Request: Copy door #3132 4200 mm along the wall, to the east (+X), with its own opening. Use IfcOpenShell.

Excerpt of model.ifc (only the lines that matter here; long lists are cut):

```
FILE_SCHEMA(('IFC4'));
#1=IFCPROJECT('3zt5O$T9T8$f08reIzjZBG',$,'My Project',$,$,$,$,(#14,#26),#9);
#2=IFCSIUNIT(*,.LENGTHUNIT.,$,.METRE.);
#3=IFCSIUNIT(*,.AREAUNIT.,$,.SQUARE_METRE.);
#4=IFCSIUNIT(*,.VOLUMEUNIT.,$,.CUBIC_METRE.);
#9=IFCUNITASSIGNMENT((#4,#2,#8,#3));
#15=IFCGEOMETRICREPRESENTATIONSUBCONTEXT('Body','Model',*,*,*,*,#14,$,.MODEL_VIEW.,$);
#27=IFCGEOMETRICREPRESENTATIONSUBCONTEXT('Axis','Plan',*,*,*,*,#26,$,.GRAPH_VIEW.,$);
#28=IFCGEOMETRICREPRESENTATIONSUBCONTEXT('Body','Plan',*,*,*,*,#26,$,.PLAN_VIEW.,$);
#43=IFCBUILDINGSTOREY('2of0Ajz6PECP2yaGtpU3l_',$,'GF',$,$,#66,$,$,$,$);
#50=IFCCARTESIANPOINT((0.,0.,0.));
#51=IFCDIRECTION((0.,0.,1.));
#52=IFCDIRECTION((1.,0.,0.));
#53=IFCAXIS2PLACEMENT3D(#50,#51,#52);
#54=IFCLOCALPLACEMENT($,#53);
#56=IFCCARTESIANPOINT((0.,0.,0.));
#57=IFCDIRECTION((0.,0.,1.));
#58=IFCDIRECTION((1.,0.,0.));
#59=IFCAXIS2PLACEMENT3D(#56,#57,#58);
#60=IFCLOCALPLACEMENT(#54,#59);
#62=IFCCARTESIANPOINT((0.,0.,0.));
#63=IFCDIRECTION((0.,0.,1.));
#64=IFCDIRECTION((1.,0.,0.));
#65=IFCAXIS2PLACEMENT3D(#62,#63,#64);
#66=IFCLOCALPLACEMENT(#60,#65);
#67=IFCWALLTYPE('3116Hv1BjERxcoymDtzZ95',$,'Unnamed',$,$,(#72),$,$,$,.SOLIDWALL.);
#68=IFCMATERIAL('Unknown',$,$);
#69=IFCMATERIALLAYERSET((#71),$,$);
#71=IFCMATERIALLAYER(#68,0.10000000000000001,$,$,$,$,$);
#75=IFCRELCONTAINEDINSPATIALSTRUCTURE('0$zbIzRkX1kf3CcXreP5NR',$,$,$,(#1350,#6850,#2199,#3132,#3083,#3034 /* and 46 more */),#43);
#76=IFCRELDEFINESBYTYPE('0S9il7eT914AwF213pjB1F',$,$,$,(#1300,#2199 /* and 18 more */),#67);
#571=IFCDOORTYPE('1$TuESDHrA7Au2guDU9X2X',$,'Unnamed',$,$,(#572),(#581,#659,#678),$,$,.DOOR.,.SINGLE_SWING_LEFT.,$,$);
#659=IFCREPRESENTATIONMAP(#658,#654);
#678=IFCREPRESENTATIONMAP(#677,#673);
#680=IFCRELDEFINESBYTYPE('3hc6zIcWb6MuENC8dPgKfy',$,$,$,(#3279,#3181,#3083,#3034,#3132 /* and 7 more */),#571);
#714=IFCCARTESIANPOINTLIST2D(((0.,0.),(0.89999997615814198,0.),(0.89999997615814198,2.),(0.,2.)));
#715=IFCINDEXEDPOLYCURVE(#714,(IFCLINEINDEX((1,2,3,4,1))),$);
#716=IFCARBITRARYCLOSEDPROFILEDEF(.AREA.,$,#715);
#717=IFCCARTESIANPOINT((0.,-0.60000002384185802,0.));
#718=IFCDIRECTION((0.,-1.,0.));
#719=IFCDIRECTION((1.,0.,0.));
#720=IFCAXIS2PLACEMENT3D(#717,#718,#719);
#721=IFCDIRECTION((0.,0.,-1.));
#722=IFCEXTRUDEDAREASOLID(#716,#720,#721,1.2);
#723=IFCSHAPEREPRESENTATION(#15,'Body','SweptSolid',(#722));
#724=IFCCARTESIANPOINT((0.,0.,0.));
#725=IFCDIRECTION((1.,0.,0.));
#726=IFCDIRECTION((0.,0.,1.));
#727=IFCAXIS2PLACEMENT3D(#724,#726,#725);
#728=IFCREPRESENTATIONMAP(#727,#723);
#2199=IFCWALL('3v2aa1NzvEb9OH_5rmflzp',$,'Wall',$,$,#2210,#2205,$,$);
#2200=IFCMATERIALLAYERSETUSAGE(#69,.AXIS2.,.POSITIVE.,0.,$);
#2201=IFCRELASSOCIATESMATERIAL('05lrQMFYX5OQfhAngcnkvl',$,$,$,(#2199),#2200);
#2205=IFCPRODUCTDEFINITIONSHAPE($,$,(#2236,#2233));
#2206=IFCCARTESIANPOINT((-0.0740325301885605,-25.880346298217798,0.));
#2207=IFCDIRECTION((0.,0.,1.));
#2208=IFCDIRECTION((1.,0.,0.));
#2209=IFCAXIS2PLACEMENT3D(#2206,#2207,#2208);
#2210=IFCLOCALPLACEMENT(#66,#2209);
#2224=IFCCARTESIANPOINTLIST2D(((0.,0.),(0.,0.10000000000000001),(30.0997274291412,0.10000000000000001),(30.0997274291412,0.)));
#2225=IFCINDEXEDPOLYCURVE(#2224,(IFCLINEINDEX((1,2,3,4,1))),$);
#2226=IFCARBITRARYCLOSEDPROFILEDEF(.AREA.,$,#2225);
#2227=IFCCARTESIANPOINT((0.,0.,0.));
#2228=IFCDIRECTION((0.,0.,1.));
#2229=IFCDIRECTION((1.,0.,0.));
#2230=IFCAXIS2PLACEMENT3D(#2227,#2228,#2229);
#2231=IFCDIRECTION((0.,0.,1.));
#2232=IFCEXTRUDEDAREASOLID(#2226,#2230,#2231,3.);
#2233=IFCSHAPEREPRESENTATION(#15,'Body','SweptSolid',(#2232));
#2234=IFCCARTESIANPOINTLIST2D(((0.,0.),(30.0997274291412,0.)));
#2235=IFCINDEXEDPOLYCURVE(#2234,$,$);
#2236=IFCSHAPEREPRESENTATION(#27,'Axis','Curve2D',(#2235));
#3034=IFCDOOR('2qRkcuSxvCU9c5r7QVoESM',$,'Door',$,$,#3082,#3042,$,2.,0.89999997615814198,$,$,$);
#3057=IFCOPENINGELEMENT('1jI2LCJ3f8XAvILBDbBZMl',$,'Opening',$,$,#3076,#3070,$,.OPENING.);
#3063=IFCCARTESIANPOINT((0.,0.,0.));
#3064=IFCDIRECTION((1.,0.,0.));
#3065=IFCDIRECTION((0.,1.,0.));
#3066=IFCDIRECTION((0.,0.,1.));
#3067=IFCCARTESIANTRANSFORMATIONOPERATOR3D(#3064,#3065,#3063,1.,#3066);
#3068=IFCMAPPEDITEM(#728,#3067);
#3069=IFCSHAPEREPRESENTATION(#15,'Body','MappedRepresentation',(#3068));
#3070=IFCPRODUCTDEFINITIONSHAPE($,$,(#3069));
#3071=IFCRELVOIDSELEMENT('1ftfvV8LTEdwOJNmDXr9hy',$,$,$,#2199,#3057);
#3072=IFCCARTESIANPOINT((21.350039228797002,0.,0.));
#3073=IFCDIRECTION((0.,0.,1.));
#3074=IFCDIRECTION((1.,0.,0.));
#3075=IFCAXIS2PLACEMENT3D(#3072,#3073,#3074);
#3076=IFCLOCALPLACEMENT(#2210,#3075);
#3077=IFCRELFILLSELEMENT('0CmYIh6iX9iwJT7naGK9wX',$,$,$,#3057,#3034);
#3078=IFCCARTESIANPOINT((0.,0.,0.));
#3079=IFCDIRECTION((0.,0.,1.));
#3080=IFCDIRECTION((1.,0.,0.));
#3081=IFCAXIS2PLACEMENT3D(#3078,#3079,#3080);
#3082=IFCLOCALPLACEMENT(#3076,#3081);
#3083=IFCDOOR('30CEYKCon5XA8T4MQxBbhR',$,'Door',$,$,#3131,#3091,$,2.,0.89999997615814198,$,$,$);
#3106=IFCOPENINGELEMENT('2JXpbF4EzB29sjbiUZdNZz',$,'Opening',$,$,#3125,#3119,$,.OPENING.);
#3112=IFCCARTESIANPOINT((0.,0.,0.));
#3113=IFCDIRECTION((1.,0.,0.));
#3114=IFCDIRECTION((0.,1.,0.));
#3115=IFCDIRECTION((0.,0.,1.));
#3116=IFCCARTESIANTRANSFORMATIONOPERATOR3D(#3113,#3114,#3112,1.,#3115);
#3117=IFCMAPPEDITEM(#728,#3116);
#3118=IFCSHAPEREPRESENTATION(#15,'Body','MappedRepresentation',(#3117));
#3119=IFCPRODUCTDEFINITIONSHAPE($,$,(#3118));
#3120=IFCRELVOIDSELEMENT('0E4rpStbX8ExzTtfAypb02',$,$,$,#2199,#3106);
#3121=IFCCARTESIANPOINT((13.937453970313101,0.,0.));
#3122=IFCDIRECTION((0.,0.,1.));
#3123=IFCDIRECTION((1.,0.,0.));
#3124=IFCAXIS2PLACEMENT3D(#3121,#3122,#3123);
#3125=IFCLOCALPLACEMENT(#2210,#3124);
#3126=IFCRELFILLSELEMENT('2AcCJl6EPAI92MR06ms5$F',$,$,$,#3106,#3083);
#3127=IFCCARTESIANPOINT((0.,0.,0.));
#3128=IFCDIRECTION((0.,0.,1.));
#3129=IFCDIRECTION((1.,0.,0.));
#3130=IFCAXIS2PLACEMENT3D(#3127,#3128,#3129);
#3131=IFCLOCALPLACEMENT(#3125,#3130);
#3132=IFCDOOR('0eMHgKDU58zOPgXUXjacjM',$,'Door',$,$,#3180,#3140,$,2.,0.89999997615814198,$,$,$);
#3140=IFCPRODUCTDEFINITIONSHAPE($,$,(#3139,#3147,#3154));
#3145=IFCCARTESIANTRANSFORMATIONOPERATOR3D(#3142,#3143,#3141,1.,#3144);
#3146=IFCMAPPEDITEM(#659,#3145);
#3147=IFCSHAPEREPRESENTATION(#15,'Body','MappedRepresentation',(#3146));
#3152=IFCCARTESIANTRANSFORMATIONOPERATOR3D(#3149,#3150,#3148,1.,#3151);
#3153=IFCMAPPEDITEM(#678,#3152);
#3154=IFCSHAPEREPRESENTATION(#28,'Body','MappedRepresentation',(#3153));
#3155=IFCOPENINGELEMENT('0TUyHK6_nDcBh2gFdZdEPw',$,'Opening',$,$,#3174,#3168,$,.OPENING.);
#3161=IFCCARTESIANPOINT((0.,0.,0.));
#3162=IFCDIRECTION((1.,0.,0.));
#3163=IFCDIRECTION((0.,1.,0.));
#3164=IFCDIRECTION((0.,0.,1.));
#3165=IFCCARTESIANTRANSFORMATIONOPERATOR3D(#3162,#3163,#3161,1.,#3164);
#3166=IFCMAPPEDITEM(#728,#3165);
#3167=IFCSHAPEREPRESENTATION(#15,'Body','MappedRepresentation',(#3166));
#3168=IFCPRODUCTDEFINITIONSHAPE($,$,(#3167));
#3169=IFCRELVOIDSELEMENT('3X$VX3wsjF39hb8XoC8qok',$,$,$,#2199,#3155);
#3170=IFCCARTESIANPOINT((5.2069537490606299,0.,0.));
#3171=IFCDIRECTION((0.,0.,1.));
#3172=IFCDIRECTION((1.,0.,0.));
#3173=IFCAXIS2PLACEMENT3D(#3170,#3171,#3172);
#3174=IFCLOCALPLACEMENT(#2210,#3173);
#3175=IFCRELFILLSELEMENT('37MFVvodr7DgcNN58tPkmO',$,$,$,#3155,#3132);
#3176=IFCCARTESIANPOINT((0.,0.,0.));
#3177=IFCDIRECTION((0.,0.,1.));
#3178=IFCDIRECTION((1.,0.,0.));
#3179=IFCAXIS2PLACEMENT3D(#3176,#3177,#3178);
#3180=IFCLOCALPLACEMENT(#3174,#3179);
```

```python
import ifcopenshell
import ifcopenshell.api.feature
import ifcopenshell.api.geometry
import ifcopenshell.api.root
import ifcopenshell.geom
import ifcopenshell.util.element
import ifcopenshell.util.placement
import ifcopenshell.util.shape
import ifcopenshell.util.unit

model = ifcopenshell.open("model.ifc")
unit_scale = ifcopenshell.util.unit.calculate_unit_scale(model)
settings = ifcopenshell.geom.settings()


def volume(element):
    """Net volume in cubic metres, openings subtracted."""
    shape = ifcopenshell.geom.create_shape(settings, element)
    return ifcopenshell.util.shape.get_volume(shape.geometry)


door = model.by_id(3132)
opening = door.FillsVoids[0].RelatingOpeningElement
wall = opening.VoidsElements[0].RelatingBuildingElement
before = volume(wall)
shift = ifcopenshell.util.placement.get_local_placement(wall.ObjectPlacement)[:3, 0] * 4.2 / unit_scale

# copy_class copies the void relationship, type, container and properties, but no geometry.
new_opening = ifcopenshell.api.root.copy_class(model, product=opening)
new_opening.Representation = ifcopenshell.util.element.copy_deep(
    model, opening.Representation, exclude=["IfcGeometricRepresentationContext", "IfcRepresentationMap"]
)
new_door = ifcopenshell.api.root.copy_class(model, product=door)
new_door.Representation = ifcopenshell.util.element.copy_deep(
    model, door.Representation, exclude=["IfcGeometricRepresentationContext", "IfcRepresentationMap"]
)
ifcopenshell.api.feature.add_filling(model, opening=new_opening, element=new_door)

for old, new in ((opening, new_opening), (door, new_door)):
    matrix = ifcopenshell.util.placement.get_local_placement(old.ObjectPlacement)
    matrix[:3, 3] += shift
    ifcopenshell.api.geometry.edit_object_placement(model, product=new, matrix=matrix, is_si=False)

after = volume(wall)

print(f"wall volume {before:.3f} -> {after:.3f} m3")

model.write("model_edited.ifc")
```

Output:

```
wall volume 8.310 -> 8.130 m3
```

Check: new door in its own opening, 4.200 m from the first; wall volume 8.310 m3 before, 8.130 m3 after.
